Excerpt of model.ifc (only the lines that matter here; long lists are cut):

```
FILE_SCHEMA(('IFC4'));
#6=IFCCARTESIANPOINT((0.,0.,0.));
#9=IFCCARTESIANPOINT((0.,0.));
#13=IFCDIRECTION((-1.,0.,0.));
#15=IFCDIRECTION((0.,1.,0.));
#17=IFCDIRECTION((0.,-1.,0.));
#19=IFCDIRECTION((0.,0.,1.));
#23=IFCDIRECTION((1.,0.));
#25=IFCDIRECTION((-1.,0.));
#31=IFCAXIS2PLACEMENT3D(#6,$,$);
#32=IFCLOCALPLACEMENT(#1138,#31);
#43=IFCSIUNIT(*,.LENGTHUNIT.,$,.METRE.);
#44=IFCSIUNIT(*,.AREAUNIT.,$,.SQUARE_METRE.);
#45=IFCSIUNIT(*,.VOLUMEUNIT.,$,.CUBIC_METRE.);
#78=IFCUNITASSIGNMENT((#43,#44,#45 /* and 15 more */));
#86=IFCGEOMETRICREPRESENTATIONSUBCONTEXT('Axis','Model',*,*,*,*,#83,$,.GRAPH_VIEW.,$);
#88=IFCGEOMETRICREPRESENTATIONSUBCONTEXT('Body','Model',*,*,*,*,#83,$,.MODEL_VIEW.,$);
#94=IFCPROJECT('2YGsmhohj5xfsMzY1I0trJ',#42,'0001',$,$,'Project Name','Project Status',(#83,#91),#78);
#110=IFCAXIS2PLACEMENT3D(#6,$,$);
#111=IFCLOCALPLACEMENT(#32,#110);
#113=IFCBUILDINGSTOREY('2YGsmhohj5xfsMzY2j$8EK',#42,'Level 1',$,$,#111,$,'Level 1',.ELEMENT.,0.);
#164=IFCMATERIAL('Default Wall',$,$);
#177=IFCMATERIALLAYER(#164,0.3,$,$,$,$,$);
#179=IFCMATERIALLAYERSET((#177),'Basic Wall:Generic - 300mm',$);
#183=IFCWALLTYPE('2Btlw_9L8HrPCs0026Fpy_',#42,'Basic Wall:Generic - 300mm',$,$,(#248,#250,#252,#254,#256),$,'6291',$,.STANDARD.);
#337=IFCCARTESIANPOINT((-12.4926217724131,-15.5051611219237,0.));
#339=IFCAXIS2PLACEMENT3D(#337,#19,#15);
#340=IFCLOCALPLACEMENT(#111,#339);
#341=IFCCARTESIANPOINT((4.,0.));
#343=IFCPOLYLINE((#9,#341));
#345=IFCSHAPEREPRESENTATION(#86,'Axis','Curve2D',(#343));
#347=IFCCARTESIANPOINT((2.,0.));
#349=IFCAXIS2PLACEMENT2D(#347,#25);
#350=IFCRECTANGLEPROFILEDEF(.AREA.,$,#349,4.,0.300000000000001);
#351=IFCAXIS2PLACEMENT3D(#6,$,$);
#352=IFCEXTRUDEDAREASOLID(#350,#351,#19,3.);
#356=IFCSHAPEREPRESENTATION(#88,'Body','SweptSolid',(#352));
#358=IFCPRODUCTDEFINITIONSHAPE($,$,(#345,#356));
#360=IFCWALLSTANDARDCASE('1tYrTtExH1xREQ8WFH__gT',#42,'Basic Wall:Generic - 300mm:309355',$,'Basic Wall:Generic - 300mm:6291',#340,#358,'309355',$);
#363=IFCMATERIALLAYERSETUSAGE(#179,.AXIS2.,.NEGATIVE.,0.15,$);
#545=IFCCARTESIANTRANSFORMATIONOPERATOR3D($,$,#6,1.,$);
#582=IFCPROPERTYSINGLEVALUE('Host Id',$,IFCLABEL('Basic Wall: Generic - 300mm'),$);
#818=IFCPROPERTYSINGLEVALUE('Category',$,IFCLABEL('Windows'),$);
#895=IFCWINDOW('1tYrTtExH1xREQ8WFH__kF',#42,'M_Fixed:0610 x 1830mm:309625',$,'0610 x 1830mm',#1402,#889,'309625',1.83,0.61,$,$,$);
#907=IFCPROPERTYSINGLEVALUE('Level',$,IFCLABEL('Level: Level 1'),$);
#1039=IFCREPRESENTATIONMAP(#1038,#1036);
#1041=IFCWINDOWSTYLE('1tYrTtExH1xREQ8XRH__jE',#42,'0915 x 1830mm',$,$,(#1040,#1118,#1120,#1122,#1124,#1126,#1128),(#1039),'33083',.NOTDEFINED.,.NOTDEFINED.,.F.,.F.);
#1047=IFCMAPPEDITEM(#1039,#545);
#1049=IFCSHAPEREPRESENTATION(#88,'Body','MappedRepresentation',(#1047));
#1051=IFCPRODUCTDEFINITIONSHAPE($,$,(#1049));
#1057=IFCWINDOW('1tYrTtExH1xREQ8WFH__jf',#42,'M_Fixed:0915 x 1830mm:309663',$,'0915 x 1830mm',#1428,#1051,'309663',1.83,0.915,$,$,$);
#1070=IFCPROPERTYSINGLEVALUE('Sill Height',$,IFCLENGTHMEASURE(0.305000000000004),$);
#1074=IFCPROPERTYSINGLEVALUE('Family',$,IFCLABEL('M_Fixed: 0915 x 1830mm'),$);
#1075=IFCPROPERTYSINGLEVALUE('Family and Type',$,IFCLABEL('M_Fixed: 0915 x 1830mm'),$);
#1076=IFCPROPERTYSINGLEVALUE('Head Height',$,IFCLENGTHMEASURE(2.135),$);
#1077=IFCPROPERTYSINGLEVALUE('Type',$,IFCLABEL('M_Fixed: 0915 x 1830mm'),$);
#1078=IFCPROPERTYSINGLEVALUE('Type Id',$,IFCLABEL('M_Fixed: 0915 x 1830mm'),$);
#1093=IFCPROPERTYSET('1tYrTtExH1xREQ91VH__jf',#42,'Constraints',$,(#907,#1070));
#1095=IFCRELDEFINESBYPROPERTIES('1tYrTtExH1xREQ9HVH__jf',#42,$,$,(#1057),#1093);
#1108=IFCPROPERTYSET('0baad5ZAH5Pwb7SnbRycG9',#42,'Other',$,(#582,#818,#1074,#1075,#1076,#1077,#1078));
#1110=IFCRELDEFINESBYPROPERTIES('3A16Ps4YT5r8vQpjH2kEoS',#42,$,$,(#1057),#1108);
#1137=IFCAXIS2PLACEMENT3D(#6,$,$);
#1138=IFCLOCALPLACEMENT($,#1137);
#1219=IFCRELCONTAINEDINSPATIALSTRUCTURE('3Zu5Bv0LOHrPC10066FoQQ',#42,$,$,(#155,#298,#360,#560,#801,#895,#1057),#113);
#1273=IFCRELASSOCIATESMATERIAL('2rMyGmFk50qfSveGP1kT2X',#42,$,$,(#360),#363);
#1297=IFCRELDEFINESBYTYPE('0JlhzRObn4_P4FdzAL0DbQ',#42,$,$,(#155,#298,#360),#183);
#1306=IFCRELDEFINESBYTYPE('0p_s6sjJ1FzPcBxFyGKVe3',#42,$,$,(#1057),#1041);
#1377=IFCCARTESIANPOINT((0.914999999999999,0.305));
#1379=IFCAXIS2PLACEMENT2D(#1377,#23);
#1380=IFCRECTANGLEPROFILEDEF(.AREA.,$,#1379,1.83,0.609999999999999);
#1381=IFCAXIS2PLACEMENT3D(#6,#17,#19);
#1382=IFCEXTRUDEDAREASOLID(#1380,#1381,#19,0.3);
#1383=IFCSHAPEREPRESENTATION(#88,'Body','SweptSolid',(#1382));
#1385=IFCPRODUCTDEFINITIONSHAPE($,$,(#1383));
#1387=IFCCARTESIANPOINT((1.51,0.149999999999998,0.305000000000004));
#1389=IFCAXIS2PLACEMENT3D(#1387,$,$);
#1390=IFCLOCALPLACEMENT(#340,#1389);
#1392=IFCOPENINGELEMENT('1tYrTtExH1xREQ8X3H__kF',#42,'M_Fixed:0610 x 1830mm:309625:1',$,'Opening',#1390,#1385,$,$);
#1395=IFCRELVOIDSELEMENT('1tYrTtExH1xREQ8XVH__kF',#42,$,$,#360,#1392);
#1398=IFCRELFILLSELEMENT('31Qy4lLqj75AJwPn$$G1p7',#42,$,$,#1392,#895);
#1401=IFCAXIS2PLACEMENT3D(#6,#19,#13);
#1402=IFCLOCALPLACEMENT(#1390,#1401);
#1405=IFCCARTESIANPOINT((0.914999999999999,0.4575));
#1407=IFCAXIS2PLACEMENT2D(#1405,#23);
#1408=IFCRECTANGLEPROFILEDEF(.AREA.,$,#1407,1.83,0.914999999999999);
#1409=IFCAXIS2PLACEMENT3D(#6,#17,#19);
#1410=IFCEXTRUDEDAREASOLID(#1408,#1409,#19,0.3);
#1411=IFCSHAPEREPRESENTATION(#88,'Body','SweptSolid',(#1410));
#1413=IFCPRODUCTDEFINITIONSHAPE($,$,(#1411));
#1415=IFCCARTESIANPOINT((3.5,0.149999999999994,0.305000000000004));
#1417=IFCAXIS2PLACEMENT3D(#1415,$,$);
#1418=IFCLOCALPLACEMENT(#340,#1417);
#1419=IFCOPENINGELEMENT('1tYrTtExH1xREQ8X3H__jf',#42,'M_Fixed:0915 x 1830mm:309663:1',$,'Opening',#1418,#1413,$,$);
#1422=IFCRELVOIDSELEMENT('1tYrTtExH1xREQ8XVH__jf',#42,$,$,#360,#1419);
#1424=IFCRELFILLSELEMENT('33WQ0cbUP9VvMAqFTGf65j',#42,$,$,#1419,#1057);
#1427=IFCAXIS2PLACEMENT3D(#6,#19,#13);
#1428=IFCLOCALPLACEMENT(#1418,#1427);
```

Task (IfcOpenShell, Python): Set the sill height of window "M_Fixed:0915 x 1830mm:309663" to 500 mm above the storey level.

```python
import numpy as np
import ifcopenshell
import ifcopenshell.api.geometry
import ifcopenshell.api.pset
import ifcopenshell.geom
import ifcopenshell.util.element
import ifcopenshell.util.placement
import ifcopenshell.util.shape
import ifcopenshell.util.unit

model = ifcopenshell.open("model.ifc")
unit_scale = ifcopenshell.util.unit.calculate_unit_scale(model)

window = model.by_guid("1tYrTtExH1xREQ8WFH__jf")
opening = window.FillsVoids[0].RelatingOpeningElement
storey = ifcopenshell.util.element.get_container(window, ifc_class="IfcBuildingStorey")
level = ifcopenshell.util.placement.get_local_placement(storey.ObjectPlacement)[2, 3]

# The opening's origin need not be at the sill, so measure its lowest point.
shape = ifcopenshell.geom.create_shape(ifcopenshell.geom.settings(), opening)
bottom = ifcopenshell.util.shape.get_shape_bottom_elevation(shape, shape.geometry) / unit_scale
dz = level + 0.5 / unit_scale - bottom

shift = np.array([0.0, 0.0, dz])
# The window is placed relative to its opening, so it follows when the opening moves.
matrix = ifcopenshell.util.placement.get_local_placement(opening.ObjectPlacement)
matrix[:3, 3] += shift
ifcopenshell.api.geometry.edit_object_placement(
    model, product=opening, matrix=matrix, is_si=False, should_transform_children=True
)

# Keep the stored heights in step.
pset = model.by_id(ifcopenshell.util.element.get_pset(window, "Constraints", should_inherit=False)["id"])
ifcopenshell.api.pset.edit_pset(model, pset=pset, properties={
    "Sill Height": model.create_entity("IfcLengthMeasure", ifcopenshell.util.element.get_pset(window, "Constraints", "Sill Height") + dz),
})
pset = model.by_id(ifcopenshell.util.element.get_pset(window, "Other", should_inherit=False)["id"])
ifcopenshell.api.pset.edit_pset(model, pset=pset, properties={
    "Head Height": model.create_entity("IfcLengthMeasure", ifcopenshell.util.element.get_pset(window, "Other", "Head Height") + dz),
})

print(f"moved by {dz * unit_scale:+.3f} m")

model.write("model_edited.ifc")
```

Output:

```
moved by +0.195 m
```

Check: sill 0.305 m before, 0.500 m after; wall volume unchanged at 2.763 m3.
